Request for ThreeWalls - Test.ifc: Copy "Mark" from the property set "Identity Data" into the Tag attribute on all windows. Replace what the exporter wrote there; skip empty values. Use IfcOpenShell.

First a look at what the model holds.

```python
import ifcopenshell
import ifcopenshell.util.element

model = ifcopenshell.open("ThreeWalls - Test.ifc")
print(model.schema)
windows = model.by_type("IfcWindow")
print(len(windows), "windows")
for e in windows[:8]:
    source = ifcopenshell.util.element.get_pset(e, "Identity Data", "Mark")
    target = e.Tag
    print(e.id(), repr(source), repr(target), sep=" | ")
```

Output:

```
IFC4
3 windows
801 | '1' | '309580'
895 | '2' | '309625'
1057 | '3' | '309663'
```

```python
import ifcopenshell
import ifcopenshell.util.element

model = ifcopenshell.open("ThreeWalls - Test.ifc")

count = 0
for e in model.by_type("IfcWindow"):
    value = ifcopenshell.util.element.get_pset(e, "Identity Data", "Mark")
    current = e.Tag
    if not value or not value.strip() or current == value:
        continue
    e.Tag = value
    count += 1

print(count, "windows updated")

model.write("ThreeWalls - Test_rev.ifc")
```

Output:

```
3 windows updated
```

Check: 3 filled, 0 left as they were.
